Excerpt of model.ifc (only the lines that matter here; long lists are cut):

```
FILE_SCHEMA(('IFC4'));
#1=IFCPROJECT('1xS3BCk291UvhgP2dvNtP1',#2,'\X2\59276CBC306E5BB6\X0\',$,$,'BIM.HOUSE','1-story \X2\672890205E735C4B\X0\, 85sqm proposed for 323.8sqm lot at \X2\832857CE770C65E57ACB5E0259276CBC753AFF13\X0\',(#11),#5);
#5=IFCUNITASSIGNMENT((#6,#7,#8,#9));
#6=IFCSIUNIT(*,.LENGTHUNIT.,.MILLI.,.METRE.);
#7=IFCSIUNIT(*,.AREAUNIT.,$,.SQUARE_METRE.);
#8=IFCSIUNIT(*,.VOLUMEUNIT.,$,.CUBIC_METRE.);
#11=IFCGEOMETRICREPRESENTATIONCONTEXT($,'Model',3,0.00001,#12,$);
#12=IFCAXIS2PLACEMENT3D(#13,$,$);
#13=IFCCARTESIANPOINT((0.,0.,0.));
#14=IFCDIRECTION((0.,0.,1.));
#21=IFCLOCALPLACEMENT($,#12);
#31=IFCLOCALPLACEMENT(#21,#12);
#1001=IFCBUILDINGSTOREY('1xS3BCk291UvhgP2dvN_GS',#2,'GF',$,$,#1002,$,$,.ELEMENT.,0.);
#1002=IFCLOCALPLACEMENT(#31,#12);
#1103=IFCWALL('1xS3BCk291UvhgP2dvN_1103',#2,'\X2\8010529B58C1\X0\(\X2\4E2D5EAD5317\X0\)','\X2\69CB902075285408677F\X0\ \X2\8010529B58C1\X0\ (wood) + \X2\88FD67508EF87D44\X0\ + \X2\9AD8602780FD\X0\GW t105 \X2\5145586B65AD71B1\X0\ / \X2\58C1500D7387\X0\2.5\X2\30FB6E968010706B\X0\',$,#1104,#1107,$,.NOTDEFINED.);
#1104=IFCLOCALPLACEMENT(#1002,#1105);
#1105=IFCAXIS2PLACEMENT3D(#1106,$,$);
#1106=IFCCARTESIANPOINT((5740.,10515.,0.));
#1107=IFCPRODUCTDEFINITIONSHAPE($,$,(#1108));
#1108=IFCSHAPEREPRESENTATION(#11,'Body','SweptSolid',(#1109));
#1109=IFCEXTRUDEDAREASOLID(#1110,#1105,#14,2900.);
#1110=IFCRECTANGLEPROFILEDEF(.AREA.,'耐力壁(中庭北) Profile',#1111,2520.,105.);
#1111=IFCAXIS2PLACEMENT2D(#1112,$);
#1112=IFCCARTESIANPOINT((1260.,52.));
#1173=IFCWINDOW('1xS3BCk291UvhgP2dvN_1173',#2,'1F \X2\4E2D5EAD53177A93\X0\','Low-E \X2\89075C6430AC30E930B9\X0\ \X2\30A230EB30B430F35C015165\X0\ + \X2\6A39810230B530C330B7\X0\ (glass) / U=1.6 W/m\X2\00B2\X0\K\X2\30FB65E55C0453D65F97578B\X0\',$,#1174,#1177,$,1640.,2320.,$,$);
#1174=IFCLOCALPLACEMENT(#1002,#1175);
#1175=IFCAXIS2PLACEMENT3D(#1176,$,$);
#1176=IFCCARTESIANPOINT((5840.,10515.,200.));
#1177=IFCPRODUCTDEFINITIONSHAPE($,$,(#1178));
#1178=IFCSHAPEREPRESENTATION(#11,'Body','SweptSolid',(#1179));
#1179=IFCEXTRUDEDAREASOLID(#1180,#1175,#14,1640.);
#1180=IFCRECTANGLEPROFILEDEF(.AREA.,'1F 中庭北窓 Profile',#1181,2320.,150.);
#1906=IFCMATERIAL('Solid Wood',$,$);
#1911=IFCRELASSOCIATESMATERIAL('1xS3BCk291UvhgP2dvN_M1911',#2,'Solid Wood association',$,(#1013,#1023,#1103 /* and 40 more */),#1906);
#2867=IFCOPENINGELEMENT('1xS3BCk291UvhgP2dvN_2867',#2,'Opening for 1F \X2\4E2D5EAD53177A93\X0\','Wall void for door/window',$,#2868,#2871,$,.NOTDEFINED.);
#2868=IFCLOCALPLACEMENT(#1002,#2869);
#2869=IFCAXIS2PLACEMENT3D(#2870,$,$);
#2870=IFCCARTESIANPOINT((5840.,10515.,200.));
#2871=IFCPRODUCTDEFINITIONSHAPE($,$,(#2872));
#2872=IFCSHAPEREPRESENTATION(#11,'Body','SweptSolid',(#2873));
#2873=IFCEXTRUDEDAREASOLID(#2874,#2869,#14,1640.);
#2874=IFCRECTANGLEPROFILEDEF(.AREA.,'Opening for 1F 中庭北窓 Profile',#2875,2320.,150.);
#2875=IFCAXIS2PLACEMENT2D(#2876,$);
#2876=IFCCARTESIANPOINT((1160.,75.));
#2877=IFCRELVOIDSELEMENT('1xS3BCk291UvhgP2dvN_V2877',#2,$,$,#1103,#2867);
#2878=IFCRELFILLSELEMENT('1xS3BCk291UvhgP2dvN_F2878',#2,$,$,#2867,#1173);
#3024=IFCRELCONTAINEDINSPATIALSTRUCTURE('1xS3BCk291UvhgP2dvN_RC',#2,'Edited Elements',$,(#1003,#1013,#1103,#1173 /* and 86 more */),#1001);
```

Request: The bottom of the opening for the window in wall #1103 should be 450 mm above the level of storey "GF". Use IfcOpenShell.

```python
import numpy as np
import ifcopenshell
import ifcopenshell.api.geometry
import ifcopenshell.geom
import ifcopenshell.util.element
import ifcopenshell.util.placement
import ifcopenshell.util.shape
import ifcopenshell.util.unit

model = ifcopenshell.open("model.ifc")
unit_scale = ifcopenshell.util.unit.calculate_unit_scale(model)

window = model.by_guid("1xS3BCk291UvhgP2dvN_1173")
opening = window.FillsVoids[0].RelatingOpeningElement
storey = ifcopenshell.util.element.get_container(window, ifc_class="IfcBuildingStorey")
level = ifcopenshell.util.placement.get_local_placement(storey.ObjectPlacement)[2, 3]

# The opening's origin need not be at the sill, so measure its lowest point.
shape = ifcopenshell.geom.create_shape(ifcopenshell.geom.settings(), opening)
bottom = ifcopenshell.util.shape.get_shape_bottom_elevation(shape, shape.geometry) / unit_scale
dz = level + 450.0 - bottom

shift = np.array([0.0, 0.0, dz])
# The window is not placed relative to its opening, so move both.
for product in (opening, window):
    matrix = ifcopenshell.util.placement.get_local_placement(product.ObjectPlacement)
    matrix[:3, 3] += shift
    ifcopenshell.api.geometry.edit_object_placement(model, product=product, matrix=matrix, is_si=False)

print(f"moved by {dz * unit_scale:+.3f} m")

model.write("model_edited.ifc")
```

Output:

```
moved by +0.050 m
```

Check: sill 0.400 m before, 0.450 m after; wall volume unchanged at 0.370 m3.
